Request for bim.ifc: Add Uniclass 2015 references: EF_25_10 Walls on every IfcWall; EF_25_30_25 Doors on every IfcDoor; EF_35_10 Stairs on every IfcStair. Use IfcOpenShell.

First a look at what the model holds.

```python
import ifcopenshell

model = ifcopenshell.open("bim.ifc")
print(model.schema)
print("classifications:", [c.Name for c in model.by_type("IfcClassification")])
for ifc_class in ("IfcDoor", "IfcRoof", "IfcStair", "IfcWall", "IfcWindow"):
    print(ifc_class, len(model.by_type(ifc_class)))
```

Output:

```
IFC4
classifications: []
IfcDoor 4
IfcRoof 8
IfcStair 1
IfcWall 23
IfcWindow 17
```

```python
import ifcopenshell
import ifcopenshell.api.classification

model = ifcopenshell.open("bim.ifc")

system = ifcopenshell.api.classification.add_classification(model, classification="Uniclass 2015")

codes = {
    "IfcWall": ("EF_25_10", "Walls"),
    "IfcDoor": ("EF_25_30_25", "Doors"),
    "IfcStair": ("EF_35_10", "Stairs"),
}
for ifc_class, (code, name) in codes.items():
    products = model.by_type(ifc_class)
    ifcopenshell.api.classification.add_reference(
        model, products=products, classification=system, identification=code, name=name
    )
    print(code, len(products))

model.write("bim-out.ifc")
```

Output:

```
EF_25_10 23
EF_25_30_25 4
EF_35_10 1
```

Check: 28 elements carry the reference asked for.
